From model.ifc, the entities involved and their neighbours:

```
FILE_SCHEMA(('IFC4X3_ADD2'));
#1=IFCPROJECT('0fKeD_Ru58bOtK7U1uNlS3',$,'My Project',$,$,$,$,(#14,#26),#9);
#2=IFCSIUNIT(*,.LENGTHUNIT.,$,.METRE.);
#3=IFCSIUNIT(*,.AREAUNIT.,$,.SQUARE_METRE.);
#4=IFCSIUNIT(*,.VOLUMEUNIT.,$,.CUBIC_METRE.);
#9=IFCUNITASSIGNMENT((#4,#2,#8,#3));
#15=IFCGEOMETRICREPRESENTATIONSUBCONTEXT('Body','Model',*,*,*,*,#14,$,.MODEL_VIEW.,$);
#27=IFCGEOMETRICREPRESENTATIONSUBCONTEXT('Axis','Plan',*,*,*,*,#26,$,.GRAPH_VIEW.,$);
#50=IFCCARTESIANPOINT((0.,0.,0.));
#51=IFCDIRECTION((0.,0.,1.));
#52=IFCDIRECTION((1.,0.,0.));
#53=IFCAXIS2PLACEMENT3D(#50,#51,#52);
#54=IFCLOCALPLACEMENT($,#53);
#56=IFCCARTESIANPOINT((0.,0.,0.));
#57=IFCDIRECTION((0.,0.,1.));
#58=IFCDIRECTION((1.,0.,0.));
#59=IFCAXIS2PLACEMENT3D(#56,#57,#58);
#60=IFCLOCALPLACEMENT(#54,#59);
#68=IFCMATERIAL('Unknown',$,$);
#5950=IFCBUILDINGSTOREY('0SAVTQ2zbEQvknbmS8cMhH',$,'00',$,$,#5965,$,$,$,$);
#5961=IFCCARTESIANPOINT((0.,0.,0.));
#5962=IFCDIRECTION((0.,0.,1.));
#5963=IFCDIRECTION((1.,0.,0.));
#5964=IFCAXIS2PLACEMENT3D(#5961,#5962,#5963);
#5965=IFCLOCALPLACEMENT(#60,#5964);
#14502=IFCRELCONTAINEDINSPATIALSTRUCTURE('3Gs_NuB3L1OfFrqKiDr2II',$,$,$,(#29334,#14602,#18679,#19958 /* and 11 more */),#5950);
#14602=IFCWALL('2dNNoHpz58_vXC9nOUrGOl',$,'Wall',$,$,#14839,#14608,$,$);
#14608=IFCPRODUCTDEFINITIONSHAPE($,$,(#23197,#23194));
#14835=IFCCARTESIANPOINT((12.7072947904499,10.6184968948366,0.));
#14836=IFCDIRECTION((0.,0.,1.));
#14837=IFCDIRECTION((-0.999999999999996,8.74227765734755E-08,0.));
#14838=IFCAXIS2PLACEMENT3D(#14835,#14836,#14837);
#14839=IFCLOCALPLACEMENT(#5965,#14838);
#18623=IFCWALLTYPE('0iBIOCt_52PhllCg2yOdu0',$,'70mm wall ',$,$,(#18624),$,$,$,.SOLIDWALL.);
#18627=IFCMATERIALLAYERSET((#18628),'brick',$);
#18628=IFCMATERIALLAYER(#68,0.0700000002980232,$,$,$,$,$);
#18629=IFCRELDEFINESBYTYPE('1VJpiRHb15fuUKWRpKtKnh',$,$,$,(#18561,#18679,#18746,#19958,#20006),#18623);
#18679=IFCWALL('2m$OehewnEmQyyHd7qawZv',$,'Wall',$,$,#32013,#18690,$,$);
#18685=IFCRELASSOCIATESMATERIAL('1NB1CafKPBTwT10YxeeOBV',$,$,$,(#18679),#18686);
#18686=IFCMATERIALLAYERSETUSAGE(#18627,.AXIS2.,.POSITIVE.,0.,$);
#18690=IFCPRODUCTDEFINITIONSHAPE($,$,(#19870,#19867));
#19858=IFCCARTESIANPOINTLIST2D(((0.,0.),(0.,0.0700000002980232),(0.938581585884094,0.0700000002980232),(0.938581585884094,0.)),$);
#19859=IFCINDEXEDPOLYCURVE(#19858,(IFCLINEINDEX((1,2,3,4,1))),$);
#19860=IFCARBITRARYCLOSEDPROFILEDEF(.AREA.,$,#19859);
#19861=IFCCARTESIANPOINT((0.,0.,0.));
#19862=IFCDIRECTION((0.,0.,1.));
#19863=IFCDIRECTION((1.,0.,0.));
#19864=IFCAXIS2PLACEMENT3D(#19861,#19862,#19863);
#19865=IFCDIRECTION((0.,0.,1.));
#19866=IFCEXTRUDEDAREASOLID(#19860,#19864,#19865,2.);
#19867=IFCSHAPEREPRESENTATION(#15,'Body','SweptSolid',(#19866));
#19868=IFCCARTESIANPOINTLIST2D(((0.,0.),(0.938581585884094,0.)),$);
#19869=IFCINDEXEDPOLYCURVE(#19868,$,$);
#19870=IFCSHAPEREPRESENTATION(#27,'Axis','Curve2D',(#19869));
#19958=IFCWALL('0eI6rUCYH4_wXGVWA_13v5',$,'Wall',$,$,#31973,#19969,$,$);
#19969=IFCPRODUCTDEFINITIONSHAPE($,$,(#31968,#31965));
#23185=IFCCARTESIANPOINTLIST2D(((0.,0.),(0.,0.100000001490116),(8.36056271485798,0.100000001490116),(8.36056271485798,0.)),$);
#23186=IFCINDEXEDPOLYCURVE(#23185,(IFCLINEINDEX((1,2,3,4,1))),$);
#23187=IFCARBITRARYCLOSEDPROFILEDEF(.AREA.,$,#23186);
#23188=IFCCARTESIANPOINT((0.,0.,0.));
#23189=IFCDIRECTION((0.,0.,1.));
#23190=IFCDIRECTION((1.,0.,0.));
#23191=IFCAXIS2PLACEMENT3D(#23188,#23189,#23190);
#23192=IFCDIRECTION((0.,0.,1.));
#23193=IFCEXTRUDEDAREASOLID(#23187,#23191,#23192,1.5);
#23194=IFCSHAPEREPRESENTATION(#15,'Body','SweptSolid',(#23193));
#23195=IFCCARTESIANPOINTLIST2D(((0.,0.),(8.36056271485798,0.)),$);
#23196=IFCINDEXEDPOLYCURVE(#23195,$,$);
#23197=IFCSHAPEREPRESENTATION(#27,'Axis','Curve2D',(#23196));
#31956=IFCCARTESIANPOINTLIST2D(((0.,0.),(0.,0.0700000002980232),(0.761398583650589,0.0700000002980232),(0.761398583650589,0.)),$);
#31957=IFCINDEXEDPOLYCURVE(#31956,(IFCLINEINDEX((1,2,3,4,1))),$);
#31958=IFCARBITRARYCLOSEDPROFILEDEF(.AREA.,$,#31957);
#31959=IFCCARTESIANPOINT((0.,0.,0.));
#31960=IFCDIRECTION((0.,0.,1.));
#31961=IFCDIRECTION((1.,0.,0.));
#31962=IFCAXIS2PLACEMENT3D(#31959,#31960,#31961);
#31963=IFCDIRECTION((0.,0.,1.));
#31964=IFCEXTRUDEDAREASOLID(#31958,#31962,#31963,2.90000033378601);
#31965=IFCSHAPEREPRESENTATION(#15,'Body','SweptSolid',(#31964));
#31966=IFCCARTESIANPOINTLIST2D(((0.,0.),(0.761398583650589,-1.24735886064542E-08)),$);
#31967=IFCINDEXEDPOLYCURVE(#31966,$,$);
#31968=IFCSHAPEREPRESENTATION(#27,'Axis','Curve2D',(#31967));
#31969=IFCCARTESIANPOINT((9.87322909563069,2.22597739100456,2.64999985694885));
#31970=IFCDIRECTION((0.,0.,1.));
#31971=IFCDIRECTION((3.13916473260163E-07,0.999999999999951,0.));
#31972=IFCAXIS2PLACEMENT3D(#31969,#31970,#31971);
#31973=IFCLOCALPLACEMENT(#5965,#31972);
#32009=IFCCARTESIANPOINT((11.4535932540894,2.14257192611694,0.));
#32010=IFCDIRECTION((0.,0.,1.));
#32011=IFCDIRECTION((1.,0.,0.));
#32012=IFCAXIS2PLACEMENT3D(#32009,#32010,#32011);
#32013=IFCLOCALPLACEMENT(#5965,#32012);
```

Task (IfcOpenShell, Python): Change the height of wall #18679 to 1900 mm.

```python
import ifcopenshell
import ifcopenshell.geom
import ifcopenshell.util.representation
import ifcopenshell.util.shape

model = ifcopenshell.open("model.ifc")
settings = ifcopenshell.geom.settings()


def volume(element):
    """Net volume in cubic metres, openings subtracted."""
    shape = ifcopenshell.geom.create_shape(settings, element)
    return ifcopenshell.util.shape.get_volume(shape.geometry)


wall = model.by_guid("2m$OehewnEmQyyHd7qawZv")
before = volume(wall)

body = ifcopenshell.util.representation.get_representation(wall, "Model", "Body")
solid = body.Items[0]
old_height = solid.Depth
solid.Depth = 1.9
after = volume(wall)

print(f"height {old_height:g} -> {solid.Depth:g}, volume {before:.3f} -> {after:.3f} m3")

model.write("model_v2.ifc")
```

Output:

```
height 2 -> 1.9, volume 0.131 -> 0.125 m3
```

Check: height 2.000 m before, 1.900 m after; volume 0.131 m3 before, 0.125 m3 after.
